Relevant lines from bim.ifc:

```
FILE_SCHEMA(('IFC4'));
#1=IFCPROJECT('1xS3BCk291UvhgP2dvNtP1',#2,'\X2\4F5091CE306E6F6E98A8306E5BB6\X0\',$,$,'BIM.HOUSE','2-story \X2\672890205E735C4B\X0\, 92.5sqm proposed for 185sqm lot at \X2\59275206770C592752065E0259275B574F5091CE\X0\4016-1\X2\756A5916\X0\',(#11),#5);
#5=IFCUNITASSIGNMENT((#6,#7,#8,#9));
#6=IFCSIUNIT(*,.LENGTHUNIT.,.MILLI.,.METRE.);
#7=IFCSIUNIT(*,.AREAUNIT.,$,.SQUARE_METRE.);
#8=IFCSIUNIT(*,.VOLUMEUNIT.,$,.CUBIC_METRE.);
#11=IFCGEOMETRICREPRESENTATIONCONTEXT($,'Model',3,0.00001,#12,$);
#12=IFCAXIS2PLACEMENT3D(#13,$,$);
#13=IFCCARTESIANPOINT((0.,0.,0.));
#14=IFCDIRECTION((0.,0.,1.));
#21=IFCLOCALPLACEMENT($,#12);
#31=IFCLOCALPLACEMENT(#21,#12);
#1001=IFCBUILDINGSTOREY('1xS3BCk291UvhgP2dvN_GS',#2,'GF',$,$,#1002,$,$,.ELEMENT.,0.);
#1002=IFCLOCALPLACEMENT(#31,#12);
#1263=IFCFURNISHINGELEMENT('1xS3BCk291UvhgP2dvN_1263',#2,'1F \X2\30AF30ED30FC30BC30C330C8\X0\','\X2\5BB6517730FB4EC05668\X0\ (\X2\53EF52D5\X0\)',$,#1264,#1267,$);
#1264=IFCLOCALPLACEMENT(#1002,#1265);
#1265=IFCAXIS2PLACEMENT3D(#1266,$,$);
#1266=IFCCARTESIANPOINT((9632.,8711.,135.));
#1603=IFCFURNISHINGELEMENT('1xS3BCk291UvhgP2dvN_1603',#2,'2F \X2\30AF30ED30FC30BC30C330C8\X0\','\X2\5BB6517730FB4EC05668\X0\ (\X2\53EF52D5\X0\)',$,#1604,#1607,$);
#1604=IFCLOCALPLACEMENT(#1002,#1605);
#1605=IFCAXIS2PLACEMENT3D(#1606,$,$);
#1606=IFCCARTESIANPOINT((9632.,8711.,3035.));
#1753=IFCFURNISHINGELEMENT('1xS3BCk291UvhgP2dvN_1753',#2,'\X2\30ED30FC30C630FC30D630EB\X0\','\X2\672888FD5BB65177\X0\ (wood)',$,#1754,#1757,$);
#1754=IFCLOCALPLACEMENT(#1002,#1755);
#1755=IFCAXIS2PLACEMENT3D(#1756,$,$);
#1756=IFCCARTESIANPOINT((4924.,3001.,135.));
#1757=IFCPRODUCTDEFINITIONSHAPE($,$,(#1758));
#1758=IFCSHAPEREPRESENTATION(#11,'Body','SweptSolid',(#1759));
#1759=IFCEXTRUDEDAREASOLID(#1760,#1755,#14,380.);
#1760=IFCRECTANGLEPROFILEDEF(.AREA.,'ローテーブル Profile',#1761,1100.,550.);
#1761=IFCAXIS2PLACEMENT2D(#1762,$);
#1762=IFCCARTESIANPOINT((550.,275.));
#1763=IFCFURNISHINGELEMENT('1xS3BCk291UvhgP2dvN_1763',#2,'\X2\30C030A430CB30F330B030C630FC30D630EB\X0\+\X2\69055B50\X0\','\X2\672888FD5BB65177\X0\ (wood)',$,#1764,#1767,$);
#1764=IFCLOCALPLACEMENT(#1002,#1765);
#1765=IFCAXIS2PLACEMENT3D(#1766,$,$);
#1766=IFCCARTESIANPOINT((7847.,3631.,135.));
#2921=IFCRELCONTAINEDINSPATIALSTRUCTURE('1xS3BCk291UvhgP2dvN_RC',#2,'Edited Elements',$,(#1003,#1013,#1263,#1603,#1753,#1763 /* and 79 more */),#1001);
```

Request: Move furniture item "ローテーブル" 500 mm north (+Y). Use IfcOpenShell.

```python
import ifcopenshell
import ifcopenshell.api.geometry
import ifcopenshell.util.placement
import ifcopenshell.util.unit

model = ifcopenshell.open("bim.ifc")
unit_scale = ifcopenshell.util.unit.calculate_unit_scale(model)

item = model.by_guid("1xS3BCk291UvhgP2dvN_1753")
matrix = ifcopenshell.util.placement.get_local_placement(item.ObjectPlacement)
matrix[1, 3] += 0.5 / unit_scale
ifcopenshell.api.geometry.edit_object_placement(model, product=item, matrix=matrix, is_si=False)

print(ifcopenshell.util.placement.get_local_placement(item.ObjectPlacement).round(3) + 0.0)

model.write("bim_updated.ifc")
```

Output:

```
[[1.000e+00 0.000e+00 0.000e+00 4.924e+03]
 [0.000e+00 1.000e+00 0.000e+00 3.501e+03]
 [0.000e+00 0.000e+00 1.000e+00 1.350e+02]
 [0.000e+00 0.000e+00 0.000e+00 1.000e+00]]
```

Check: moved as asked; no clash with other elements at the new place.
